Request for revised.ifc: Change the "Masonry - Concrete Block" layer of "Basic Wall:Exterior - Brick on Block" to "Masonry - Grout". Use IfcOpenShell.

First a look at what the model holds.

```python
import ifcopenshell
import ifcopenshell.util.element

model = ifcopenshell.open("revised.ifc")
print(model.schema)
for layer_set in model.by_type("IfcMaterialLayerSet"):
    if layer_set.LayerSetName == "Basic Wall:Exterior - Brick on Block":
        for layer in layer_set.MaterialLayers:
            print(layer.id(), layer.Material and layer.Material.Name, layer.LayerThickness, sep=" | ")
        print(len(ifcopenshell.util.element.get_elements_by_material(model, layer_set)), "elements and types use it")
print(sorted(m.Name for m in model.by_type("IfcMaterial") if m.Name)[:60])
```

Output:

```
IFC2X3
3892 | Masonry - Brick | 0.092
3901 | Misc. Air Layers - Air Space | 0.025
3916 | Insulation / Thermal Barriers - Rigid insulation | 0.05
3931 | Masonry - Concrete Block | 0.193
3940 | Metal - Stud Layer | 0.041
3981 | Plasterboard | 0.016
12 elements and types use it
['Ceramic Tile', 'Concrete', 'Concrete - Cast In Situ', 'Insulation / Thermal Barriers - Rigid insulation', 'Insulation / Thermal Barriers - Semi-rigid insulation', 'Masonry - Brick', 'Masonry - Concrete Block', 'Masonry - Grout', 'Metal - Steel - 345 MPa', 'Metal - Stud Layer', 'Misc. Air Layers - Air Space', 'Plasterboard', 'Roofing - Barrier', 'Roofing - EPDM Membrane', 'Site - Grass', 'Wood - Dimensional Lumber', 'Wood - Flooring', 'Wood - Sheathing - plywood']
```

```python
import ifcopenshell
import ifcopenshell.api.material

model = ifcopenshell.open("revised.ifc")

layer_set = next(s for s in model.by_type("IfcMaterialLayerSet") if s.LayerSetName == "Basic Wall:Exterior - Brick on Block")
layer = next(l for l in layer_set.MaterialLayers if l.Material and l.Material.Name == "Masonry - Concrete Block")
material = next(m for m in model.by_type("IfcMaterial") if m.Name == "Masonry - Grout")

# Point this one layer at the other material; renaming the old one would change it everywhere.
ifcopenshell.api.material.edit_layer(model, layer=layer, attributes={}, material=material)

print([l.Material.Name if l.Material else None for l in layer_set.MaterialLayers])

model.write("revised_updated.ifc")
```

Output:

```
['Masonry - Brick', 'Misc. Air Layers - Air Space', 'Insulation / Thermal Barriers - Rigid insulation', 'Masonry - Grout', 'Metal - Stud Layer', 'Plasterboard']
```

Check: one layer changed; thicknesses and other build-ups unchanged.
